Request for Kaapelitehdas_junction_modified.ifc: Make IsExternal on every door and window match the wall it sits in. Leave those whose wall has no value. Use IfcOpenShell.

First a look at what the model holds.

```python
import ifcopenshell
import ifcopenshell.util.element

model = ifcopenshell.open("Kaapelitehdas_junction_modified.ifc")
print(model.schema)
seen = {}
for e in model.by_type("IfcDoor") + model.by_type("IfcWindow"):
    if not e.FillsVoids:
        continue
    host = e.FillsVoids[0].RelatingOpeningElement.VoidsElements[0].RelatingBuildingElement
    own = ifcopenshell.util.element.get_pset(e, f"Pset_{e.is_a()[3:].removesuffix('StandardCase')}Common", "IsExternal")
    wall = ifcopenshell.util.element.get_pset(host, "Pset_WallCommon", "IsExternal")
    seen[e.is_a(), own, wall] = seen.get((e.is_a(), own, wall), 0) + 1
for (cls, own, wall), count in sorted(seen.items(), key=str):
    print(count, cls, "IsExternal:", own, "| host wall:", wall)
```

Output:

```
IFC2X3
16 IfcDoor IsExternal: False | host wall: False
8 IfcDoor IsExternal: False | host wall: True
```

```python
import ifcopenshell
import ifcopenshell.api.pset
import ifcopenshell.util.element

model = ifcopenshell.open("Kaapelitehdas_junction_modified.ifc")

count = 0
for ifc_class, pset_name in (("IfcDoor", "Pset_DoorCommon"), ("IfcWindow", "Pset_WindowCommon")):
    for e in model.by_type(ifc_class):
        if not e.FillsVoids:
            continue
        host = e.FillsVoids[0].RelatingOpeningElement.VoidsElements[0].RelatingBuildingElement
        external = ifcopenshell.util.element.get_pset(host, "Pset_WallCommon", "IsExternal")
        if external is None or ifcopenshell.util.element.get_pset(e, pset_name, "IsExternal") == external:
            continue
        pset = ifcopenshell.api.pset.add_pset(model, product=e, name=pset_name)
        ifcopenshell.api.pset.edit_pset(model, pset=pset, properties={"IsExternal": external})
        count += 1

print(count, "updated")

model.write("Kaapelitehdas_junction_modified_edited.ifc")
```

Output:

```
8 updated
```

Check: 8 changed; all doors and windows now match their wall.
